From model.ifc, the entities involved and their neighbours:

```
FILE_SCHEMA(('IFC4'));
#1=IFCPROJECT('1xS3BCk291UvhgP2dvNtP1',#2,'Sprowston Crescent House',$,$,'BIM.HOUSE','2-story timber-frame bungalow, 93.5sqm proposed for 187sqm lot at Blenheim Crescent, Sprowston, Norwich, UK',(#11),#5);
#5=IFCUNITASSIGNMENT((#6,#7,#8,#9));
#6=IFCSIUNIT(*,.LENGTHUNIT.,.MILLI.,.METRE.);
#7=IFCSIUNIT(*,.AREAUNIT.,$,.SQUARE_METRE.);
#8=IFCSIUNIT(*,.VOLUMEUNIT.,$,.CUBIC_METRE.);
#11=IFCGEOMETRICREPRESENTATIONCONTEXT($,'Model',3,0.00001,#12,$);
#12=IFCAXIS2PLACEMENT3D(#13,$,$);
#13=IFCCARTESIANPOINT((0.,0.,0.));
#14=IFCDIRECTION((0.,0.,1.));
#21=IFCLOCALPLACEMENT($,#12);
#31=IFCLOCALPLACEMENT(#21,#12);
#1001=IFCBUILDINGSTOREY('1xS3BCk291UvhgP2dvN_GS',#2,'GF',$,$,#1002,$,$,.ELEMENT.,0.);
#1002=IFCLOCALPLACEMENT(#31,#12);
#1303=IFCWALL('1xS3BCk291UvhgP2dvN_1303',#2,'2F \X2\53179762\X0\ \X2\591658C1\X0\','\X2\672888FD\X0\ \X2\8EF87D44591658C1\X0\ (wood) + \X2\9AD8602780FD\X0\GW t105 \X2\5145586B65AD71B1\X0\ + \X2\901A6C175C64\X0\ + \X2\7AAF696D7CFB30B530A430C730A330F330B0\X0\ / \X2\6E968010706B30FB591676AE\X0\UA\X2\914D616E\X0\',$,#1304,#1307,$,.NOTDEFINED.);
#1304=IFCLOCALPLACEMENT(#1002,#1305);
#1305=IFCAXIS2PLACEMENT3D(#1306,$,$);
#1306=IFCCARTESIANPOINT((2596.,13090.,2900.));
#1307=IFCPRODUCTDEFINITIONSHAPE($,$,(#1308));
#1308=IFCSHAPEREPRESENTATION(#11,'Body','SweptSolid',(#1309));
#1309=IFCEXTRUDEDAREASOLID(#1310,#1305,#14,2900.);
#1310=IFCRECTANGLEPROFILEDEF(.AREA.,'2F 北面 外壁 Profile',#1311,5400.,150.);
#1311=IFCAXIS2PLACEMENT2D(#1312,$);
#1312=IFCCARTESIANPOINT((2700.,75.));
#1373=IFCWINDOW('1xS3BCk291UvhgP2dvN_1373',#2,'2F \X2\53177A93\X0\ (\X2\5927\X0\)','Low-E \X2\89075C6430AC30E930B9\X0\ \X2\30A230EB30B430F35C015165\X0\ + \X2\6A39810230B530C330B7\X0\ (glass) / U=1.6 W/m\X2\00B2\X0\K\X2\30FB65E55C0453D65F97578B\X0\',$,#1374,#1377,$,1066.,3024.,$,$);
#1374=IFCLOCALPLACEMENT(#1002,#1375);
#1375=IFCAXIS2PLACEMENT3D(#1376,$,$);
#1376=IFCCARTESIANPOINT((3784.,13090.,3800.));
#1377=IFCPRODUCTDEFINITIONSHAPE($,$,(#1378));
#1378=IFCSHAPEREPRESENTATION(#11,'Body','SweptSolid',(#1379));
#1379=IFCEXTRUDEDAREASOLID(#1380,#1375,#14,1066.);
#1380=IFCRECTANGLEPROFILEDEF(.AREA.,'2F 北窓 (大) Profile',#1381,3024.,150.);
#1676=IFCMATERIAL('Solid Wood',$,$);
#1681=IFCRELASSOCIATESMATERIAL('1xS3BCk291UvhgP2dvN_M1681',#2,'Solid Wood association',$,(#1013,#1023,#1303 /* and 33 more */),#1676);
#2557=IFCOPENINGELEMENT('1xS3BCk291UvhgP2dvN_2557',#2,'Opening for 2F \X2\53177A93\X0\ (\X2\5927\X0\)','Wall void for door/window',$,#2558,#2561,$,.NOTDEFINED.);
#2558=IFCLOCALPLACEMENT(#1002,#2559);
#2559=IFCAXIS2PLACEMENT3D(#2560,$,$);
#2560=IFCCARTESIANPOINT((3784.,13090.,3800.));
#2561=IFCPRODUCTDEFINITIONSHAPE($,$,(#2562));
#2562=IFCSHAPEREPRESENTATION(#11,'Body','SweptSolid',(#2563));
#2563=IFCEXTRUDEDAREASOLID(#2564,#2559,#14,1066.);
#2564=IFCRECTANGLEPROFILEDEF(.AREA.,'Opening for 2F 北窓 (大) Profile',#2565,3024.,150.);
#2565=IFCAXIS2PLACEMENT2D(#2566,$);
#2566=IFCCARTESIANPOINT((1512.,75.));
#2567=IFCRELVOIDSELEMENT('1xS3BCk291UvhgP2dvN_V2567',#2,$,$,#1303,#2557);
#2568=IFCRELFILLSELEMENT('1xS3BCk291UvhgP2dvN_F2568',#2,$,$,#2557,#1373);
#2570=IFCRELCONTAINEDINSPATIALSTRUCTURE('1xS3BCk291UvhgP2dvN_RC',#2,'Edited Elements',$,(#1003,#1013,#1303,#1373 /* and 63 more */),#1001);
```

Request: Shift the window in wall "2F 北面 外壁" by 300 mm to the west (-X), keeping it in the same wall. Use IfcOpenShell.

```python
import ifcopenshell
import ifcopenshell.api.geometry
import ifcopenshell.util.placement
import ifcopenshell.util.unit

model = ifcopenshell.open("model.ifc")
unit_scale = ifcopenshell.util.unit.calculate_unit_scale(model)

window = model.by_id(1373)
opening = window.FillsVoids[0].RelatingOpeningElement
wall = opening.VoidsElements[0].RelatingBuildingElement

wall_matrix = ifcopenshell.util.placement.get_local_placement(wall.ObjectPlacement)
shift = wall_matrix[:3, 0] * -0.3 / unit_scale
before = ifcopenshell.util.placement.get_local_placement(window.ObjectPlacement)[:3, 3].copy()

# The window is not placed relative to its opening, so move both.
for product in (opening, window):
    matrix = ifcopenshell.util.placement.get_local_placement(product.ObjectPlacement)
    matrix[:3, 3] += shift
    ifcopenshell.api.geometry.edit_object_placement(model, product=product, matrix=matrix, is_si=False)

after = ifcopenshell.util.placement.get_local_placement(window.ObjectPlacement)[:3, 3]
print("window moved by", (after - before).round(3) + 0.0)

model.write("model_edited.ifc")
```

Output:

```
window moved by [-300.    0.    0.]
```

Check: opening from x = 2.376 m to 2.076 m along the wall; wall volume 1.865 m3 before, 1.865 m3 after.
